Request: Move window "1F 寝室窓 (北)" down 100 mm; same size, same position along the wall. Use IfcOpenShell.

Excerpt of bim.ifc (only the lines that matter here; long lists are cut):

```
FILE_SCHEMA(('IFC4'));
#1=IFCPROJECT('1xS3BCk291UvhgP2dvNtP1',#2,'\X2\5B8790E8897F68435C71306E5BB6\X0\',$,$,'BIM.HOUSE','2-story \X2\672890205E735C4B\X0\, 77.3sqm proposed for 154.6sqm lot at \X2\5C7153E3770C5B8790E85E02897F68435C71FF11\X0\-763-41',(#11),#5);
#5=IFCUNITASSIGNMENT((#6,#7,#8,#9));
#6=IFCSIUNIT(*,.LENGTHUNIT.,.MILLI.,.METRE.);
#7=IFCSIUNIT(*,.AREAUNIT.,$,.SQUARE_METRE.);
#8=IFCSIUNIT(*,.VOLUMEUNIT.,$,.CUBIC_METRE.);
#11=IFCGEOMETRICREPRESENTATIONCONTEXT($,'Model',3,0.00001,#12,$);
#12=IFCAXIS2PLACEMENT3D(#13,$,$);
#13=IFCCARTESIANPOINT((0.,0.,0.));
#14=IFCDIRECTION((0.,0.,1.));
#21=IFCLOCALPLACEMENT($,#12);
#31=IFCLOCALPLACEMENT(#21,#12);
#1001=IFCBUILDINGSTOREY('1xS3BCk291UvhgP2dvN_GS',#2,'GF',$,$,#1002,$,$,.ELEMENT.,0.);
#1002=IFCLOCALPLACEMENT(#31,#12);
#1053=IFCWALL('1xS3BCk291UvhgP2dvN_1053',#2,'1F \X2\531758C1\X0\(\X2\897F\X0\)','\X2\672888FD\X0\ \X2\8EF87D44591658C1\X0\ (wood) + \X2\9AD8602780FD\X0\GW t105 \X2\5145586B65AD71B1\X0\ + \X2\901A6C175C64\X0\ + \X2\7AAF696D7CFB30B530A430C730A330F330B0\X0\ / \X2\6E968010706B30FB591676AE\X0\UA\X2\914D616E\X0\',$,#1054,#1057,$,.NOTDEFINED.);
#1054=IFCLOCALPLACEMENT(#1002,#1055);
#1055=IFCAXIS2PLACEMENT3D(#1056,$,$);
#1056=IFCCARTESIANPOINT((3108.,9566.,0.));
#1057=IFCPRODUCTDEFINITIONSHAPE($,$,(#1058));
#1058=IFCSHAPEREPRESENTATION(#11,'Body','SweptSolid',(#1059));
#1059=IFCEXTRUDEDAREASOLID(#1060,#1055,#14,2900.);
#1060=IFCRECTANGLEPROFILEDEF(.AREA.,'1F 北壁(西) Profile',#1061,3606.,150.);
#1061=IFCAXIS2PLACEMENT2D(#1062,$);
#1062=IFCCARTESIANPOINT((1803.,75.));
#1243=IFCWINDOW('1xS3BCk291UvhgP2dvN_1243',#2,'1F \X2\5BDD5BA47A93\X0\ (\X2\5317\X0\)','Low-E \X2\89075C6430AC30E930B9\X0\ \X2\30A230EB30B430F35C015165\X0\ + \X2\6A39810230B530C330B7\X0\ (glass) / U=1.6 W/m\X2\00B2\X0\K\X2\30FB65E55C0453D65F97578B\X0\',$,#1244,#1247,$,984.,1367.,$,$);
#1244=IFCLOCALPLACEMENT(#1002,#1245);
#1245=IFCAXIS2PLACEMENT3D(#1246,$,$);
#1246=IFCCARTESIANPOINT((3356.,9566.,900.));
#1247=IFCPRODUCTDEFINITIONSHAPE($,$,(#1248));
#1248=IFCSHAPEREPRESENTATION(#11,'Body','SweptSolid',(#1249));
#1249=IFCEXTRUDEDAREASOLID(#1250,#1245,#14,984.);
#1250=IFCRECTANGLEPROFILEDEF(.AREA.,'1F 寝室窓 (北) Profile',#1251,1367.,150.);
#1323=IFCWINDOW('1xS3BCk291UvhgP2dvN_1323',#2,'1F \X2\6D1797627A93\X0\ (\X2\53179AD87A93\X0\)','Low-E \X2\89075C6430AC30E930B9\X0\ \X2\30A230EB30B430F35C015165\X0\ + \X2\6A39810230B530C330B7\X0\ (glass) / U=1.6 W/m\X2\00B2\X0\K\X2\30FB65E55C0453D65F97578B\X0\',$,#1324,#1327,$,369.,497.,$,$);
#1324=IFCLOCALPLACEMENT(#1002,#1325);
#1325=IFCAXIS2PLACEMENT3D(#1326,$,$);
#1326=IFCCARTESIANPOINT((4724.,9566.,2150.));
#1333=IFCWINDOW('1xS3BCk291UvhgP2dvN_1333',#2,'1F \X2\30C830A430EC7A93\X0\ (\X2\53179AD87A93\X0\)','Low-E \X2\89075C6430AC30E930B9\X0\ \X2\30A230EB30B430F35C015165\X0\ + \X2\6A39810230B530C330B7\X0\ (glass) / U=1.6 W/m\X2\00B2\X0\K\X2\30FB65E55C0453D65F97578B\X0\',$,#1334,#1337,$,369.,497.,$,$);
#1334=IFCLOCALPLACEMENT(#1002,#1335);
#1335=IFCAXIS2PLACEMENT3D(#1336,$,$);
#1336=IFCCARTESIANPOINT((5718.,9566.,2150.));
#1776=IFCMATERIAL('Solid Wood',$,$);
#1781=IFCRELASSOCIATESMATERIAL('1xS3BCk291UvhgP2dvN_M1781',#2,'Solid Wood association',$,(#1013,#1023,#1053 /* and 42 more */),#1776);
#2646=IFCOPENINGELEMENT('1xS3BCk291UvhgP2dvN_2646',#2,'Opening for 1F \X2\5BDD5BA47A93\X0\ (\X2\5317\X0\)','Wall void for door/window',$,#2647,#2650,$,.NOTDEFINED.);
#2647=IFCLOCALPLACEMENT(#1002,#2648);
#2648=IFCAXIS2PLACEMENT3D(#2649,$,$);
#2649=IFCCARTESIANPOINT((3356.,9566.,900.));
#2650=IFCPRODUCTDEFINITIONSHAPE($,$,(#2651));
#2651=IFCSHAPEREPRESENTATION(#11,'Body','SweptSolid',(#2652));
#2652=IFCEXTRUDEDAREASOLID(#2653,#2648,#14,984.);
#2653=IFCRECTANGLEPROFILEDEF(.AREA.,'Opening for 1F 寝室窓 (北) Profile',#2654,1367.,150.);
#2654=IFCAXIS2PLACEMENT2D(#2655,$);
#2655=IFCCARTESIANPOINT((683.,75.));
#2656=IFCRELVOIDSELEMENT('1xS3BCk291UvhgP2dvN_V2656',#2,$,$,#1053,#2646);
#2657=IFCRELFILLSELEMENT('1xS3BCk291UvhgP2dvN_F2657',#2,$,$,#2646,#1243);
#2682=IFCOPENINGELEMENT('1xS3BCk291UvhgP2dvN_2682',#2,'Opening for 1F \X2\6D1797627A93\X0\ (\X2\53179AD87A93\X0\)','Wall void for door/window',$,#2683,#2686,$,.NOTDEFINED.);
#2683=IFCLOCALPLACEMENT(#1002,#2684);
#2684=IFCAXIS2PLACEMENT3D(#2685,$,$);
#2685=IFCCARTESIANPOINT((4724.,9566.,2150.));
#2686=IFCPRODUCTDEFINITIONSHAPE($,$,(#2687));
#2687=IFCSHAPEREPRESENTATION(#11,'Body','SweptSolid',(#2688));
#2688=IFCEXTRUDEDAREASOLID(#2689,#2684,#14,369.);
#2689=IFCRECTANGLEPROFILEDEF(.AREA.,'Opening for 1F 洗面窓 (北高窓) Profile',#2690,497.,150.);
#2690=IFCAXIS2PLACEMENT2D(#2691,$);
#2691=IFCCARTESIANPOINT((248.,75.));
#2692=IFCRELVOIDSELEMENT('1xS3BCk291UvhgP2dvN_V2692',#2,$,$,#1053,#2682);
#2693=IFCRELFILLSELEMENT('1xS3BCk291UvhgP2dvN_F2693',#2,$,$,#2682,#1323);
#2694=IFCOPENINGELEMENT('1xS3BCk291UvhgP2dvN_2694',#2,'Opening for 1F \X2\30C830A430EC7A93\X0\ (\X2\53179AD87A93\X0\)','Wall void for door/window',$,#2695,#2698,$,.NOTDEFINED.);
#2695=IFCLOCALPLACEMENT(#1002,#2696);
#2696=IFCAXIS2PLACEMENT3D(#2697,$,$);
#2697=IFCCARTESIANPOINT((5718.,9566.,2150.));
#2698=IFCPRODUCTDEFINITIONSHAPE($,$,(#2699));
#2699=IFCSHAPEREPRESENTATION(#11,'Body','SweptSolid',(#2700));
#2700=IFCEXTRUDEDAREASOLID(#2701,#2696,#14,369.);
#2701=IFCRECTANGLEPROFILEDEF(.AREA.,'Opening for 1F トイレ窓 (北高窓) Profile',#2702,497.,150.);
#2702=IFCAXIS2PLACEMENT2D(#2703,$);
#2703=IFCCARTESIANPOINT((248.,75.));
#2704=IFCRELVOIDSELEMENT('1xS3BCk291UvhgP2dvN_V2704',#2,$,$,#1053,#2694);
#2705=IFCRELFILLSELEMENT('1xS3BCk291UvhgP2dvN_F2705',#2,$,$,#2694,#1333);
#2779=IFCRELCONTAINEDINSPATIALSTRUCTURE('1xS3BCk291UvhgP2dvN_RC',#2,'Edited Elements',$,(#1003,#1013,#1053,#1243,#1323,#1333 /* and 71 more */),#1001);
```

```python
import numpy as np
import ifcopenshell
import ifcopenshell.api.geometry
import ifcopenshell.util.placement
import ifcopenshell.util.unit

model = ifcopenshell.open("bim.ifc")
unit_scale = ifcopenshell.util.unit.calculate_unit_scale(model)

window = model.by_id(1243)
opening = window.FillsVoids[0].RelatingOpeningElement
dz = -100.0

shift = np.array([0.0, 0.0, dz])
# The window is not placed relative to its opening, so move both.
for product in (opening, window):
    matrix = ifcopenshell.util.placement.get_local_placement(product.ObjectPlacement)
    matrix[:3, 3] += shift
    ifcopenshell.api.geometry.edit_object_placement(model, product=product, matrix=matrix, is_si=False)

print(f"moved by {dz * unit_scale:+.3f} m")

model.write("bim-out.ifc")
```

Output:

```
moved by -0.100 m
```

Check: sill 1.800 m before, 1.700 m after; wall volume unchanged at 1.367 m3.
